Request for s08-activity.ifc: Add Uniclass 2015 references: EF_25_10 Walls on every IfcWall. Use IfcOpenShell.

First a look at what the model holds.

```python
import ifcopenshell

model = ifcopenshell.open("s08-activity.ifc")
print(model.schema)
print("classifications:", [c.Name for c in model.by_type("IfcClassification")])
for ifc_class in ("IfcDoor", "IfcRoof", "IfcStair", "IfcWall", "IfcWindow"):
    print(ifc_class, len(model.by_type(ifc_class)))
```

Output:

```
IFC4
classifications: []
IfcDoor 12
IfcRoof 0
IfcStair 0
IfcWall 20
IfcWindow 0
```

```python
import ifcopenshell
import ifcopenshell.api.classification

model = ifcopenshell.open("s08-activity.ifc")

system = ifcopenshell.api.classification.add_classification(model, classification="Uniclass 2015")

codes = {
    "IfcWall": ("EF_25_10", "Walls"),
}
for ifc_class, (code, name) in codes.items():
    products = model.by_type(ifc_class)
    ifcopenshell.api.classification.add_reference(
        model, products=products, classification=system, identification=code, name=name
    )
    print(code, len(products))

model.write("s08-activity_edited.ifc")
```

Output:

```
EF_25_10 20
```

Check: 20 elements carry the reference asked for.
